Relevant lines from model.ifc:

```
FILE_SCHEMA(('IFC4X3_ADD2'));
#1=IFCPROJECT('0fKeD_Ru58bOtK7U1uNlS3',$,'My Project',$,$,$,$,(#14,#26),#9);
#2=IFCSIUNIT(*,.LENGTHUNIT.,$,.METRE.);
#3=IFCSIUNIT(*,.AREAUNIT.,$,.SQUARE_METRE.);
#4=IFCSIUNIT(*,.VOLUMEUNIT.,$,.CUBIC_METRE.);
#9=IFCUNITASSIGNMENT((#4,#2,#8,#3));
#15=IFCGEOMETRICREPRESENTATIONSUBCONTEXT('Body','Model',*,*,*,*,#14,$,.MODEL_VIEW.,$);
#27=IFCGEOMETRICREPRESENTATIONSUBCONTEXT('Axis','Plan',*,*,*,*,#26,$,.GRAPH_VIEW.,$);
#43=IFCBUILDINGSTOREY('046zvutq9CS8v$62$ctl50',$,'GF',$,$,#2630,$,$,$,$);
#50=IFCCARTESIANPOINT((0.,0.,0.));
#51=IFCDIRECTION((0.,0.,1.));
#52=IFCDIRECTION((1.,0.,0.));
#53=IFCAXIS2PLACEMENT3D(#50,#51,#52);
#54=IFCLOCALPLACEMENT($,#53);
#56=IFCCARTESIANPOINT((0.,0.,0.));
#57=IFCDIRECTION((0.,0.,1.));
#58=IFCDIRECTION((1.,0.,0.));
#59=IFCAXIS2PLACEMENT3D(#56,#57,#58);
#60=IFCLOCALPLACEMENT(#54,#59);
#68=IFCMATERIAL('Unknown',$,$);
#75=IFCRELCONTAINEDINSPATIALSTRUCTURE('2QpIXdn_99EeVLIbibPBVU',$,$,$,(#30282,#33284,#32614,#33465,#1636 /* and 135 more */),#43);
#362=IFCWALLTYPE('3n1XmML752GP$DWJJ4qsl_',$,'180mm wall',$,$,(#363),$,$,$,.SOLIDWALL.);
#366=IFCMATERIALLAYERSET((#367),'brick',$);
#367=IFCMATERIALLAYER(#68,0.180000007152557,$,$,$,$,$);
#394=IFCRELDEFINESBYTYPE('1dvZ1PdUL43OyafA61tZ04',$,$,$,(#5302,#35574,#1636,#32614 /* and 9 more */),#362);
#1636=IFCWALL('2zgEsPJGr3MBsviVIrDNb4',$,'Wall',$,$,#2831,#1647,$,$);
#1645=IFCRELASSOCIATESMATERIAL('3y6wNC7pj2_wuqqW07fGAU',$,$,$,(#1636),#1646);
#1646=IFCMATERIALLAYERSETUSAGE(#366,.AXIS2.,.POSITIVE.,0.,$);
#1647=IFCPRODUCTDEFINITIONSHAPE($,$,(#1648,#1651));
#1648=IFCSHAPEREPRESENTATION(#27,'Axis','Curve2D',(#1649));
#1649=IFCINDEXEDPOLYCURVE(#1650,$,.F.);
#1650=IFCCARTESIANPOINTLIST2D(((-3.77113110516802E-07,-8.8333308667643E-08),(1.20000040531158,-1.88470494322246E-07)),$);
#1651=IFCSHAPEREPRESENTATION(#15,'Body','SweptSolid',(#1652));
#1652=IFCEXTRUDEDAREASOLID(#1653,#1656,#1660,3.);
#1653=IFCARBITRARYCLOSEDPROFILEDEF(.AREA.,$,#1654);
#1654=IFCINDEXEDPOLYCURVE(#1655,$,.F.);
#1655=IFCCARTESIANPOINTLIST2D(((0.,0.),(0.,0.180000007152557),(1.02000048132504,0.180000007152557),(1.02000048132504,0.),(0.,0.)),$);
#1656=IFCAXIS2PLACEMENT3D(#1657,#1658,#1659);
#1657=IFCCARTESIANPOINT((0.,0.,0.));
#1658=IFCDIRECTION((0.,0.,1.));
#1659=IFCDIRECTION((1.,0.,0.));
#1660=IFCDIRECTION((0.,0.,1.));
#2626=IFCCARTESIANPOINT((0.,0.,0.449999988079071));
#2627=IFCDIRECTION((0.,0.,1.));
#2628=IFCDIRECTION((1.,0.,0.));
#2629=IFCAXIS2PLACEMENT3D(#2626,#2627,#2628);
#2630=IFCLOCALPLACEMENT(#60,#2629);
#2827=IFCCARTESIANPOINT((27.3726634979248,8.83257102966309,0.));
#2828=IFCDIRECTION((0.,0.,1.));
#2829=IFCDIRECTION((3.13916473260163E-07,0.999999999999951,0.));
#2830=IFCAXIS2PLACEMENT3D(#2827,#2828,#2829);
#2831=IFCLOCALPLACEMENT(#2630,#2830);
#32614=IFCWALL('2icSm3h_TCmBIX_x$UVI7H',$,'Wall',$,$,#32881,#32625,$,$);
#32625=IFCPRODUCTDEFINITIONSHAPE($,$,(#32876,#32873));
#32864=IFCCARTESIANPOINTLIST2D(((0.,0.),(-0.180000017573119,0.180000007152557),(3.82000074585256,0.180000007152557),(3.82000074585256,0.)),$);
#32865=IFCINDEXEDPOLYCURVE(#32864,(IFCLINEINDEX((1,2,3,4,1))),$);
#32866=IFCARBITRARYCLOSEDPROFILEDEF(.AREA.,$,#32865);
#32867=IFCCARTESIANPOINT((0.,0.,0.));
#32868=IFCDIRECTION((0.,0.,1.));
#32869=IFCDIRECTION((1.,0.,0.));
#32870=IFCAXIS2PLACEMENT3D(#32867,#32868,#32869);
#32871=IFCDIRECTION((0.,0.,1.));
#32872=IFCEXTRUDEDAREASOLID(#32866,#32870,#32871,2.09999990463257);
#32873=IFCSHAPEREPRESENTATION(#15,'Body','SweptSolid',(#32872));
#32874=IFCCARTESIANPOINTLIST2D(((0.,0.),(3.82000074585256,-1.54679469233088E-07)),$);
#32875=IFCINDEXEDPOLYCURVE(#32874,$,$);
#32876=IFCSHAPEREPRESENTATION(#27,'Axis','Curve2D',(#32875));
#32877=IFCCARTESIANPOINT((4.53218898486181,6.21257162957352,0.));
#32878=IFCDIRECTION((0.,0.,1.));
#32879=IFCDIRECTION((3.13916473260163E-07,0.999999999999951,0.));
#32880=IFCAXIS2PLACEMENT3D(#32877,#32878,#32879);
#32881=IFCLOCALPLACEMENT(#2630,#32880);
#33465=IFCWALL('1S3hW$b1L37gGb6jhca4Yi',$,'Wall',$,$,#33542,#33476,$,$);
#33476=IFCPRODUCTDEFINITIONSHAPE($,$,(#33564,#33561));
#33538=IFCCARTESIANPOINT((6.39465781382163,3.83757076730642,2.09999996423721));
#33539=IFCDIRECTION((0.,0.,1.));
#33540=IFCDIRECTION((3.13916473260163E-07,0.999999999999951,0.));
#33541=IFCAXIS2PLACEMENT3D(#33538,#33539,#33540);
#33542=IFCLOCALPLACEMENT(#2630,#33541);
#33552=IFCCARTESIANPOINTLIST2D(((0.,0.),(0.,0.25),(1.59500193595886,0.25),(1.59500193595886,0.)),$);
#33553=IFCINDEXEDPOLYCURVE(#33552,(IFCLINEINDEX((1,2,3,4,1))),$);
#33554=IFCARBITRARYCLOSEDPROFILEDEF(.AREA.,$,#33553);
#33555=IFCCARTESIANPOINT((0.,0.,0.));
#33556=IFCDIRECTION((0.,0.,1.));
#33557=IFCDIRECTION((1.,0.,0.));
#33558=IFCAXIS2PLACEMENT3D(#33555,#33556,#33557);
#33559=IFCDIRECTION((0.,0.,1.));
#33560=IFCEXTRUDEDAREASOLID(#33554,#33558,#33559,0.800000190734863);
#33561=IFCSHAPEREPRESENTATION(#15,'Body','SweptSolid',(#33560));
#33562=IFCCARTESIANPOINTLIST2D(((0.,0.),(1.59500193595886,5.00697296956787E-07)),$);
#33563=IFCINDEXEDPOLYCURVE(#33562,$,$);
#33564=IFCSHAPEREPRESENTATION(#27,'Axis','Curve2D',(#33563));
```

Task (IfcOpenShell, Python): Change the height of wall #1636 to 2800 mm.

```python
import ifcopenshell
import ifcopenshell.geom
import ifcopenshell.util.representation
import ifcopenshell.util.shape

model = ifcopenshell.open("model.ifc")
settings = ifcopenshell.geom.settings()


def volume(element):
    """Net volume in cubic metres, openings subtracted."""
    shape = ifcopenshell.geom.create_shape(settings, element)
    return ifcopenshell.util.shape.get_volume(shape.geometry)


wall = model.by_guid("2zgEsPJGr3MBsviVIrDNb4")
before = volume(wall)

body = ifcopenshell.util.representation.get_representation(wall, "Model", "Body")
solid = body.Items[0]
old_height = solid.Depth
solid.Depth = 2.8
after = volume(wall)

print(f"height {old_height:g} -> {solid.Depth:g}, volume {before:.3f} -> {after:.3f} m3")

model.write("model-out.ifc")
```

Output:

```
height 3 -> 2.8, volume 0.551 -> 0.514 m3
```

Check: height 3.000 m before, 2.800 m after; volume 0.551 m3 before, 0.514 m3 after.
